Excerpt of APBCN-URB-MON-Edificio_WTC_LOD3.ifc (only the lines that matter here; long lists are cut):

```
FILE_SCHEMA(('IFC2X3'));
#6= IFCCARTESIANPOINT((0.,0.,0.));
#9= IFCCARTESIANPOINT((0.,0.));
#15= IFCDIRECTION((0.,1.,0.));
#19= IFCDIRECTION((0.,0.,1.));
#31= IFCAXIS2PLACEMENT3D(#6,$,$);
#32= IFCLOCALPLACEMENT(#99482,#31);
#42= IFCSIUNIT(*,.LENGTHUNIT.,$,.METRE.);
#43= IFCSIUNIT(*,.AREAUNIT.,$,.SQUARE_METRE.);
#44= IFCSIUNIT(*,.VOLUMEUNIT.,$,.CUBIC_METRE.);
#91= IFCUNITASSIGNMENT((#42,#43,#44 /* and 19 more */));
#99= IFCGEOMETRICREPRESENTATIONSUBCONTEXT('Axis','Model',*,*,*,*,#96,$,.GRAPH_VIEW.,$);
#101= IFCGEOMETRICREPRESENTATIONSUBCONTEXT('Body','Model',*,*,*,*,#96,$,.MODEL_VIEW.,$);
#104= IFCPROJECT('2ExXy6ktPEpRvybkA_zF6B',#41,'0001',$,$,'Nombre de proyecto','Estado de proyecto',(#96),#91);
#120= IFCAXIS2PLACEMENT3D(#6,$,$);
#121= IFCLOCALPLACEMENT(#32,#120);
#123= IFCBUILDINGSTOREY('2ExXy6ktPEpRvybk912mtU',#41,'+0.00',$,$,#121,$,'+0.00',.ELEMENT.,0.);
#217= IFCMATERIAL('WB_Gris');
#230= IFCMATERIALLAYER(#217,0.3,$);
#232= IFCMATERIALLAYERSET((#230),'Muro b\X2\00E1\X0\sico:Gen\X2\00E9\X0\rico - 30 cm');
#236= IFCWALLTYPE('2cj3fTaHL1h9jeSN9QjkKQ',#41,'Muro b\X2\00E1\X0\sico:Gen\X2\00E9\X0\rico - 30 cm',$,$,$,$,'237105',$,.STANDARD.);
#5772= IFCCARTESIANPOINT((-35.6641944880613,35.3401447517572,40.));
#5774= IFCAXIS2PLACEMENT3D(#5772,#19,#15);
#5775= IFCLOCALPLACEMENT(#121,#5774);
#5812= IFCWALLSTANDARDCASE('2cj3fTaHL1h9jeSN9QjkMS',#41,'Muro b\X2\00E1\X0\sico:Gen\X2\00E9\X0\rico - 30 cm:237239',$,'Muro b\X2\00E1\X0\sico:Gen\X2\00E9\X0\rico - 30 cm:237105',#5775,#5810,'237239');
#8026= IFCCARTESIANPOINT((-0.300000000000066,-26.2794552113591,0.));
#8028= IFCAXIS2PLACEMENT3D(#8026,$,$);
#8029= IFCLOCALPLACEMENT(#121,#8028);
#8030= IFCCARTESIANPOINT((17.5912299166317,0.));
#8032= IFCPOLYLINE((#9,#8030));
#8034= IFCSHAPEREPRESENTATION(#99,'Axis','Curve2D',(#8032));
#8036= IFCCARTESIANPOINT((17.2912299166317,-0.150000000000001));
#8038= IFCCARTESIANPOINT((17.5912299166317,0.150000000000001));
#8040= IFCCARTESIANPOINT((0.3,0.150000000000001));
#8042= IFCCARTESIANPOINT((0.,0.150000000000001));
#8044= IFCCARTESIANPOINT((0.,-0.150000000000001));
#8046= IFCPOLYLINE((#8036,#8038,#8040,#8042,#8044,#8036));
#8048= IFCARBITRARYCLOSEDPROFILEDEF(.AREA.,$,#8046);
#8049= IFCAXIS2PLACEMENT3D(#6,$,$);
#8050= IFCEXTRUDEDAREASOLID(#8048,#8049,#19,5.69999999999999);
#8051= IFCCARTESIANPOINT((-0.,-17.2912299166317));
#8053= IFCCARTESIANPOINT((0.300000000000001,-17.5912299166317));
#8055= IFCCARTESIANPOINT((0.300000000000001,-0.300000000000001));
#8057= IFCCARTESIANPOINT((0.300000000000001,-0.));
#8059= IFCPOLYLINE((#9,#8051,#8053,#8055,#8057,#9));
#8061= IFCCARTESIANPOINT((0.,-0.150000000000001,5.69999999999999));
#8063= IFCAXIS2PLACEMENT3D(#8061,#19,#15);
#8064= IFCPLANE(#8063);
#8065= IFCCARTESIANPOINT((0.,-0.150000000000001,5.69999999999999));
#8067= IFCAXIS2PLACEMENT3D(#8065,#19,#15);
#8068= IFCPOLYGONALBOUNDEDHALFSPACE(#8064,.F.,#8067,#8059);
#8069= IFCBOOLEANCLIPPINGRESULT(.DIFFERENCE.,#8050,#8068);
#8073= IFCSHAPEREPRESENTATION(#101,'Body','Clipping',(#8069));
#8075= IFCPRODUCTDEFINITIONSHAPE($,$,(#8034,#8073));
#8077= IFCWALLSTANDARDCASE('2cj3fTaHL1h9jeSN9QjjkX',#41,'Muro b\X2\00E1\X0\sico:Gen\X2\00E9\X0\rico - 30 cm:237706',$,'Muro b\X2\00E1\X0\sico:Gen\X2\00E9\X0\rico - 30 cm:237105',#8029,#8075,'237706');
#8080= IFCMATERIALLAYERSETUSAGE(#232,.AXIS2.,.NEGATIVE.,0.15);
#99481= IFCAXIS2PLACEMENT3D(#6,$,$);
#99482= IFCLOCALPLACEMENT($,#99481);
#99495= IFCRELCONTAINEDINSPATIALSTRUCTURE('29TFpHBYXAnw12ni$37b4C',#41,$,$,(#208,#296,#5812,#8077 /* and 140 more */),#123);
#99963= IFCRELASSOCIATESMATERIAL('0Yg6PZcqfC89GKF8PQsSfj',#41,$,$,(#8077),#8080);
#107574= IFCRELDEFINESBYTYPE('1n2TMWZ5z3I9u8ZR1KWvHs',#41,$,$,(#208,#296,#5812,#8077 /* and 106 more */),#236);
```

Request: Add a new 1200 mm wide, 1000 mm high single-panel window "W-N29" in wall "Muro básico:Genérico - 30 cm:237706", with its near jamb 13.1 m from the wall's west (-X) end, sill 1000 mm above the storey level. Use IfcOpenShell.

```python
import numpy as np
import ifcopenshell
import ifcopenshell.api.feature
import ifcopenshell.api.geometry
import ifcopenshell.api.root
import ifcopenshell.api.spatial
import ifcopenshell.api.type
import ifcopenshell.geom
import ifcopenshell.util.element
import ifcopenshell.util.placement
import ifcopenshell.util.representation
import ifcopenshell.util.shape
import ifcopenshell.util.unit

model = ifcopenshell.open("APBCN-URB-MON-Edificio_WTC_LOD3.ifc")
unit_scale = ifcopenshell.util.unit.calculate_unit_scale(model)
settings = ifcopenshell.geom.settings()


def volume(element):
    """Net volume in cubic metres, openings subtracted."""
    shape = ifcopenshell.geom.create_shape(settings, element)
    return ifcopenshell.util.shape.get_volume(shape.geometry)


wall = model.by_guid("2cj3fTaHL1h9jeSN9QjjkX")
storey = ifcopenshell.util.element.get_container(wall, ifc_class="IfcBuildingStorey")
context = ifcopenshell.util.representation.get_context(model, "Model", "Body", "MODEL_VIEW")
before = volume(wall)

width, height, from_end, sill = 1.2, 1, 13.1, 1  # metres

# The wall runs along its own X axis, and the end named is its -X end.
wall_shape = ifcopenshell.geom.create_shape(settings, wall)
x, y, z = ifcopenshell.util.shape.get_vertices(wall_shape.geometry).T
start = x.min() + from_end
face, thickness = float(y.min()), float(y.max() - y.min())
wall_matrix = ifcopenshell.util.placement.get_local_placement(wall.ObjectPlacement)
level = ifcopenshell.util.placement.get_local_placement(storey.ObjectPlacement)[2, 3]


def in_wall(x, y):
    """Placement at x, y metres in the wall's axes, at sill height."""
    matrix = wall_matrix.copy()
    matrix[:, 3] = wall_matrix @ np.array([x / unit_scale, y / unit_scale, 0.0, 1.0])
    matrix[2, 3] = level + sill / unit_scale
    return matrix


# Opening: a box that overshoots both wall faces by 50 mm.
opening = ifcopenshell.api.root.create_entity(model, ifc_class="IfcOpeningElement")
box = ifcopenshell.api.geometry.add_wall_representation(
    model, context=context, length=width, height=height, thickness=thickness + 0.1
)
ifcopenshell.api.geometry.assign_representation(model, product=opening, representation=box)
ifcopenshell.api.geometry.edit_object_placement(model, product=opening, matrix=in_wall(start, face - 0.05), is_si=False)
ifcopenshell.api.feature.add_feature(model, feature=opening, element=wall)

window = ifcopenshell.api.root.create_entity(model, ifc_class="IfcWindow", name="W-N29")
window.OverallWidth, window.OverallHeight = width / unit_scale, height / unit_scale
body = ifcopenshell.api.geometry.add_window_representation(
    model,
    context=context,
    overall_width=window.OverallWidth,
    overall_height=window.OverallHeight,
    partition_type="SINGLE_PANEL",
)
ifcopenshell.api.geometry.assign_representation(model, product=window, representation=body)
ifcopenshell.api.spatial.assign_container(model, products=[window], relating_structure=storey)
fills = ifcopenshell.api.feature.add_filling(model, opening=opening, element=window)
fills.OwnerHistory = window.OwnerHistory  # required in IFC2X3

# IFC2X3 keeps the operation on the window style.
style = ifcopenshell.api.root.create_entity(model, ifc_class="IfcWindowStyle", name="W-N29")
style.OperationType, style.ConstructionType = "SINGLE_PANEL", "NOTDEFINED"
style.ParameterTakesPrecedence = style.Sizeable = False
ifcopenshell.api.type.assign_type(model, related_objects=[window], relating_type=style)

# Centre the window in the wall's thickness.
ifcopenshell.api.geometry.edit_object_placement(model, product=window, matrix=in_wall(start, face), is_si=False)
window_shape = ifcopenshell.geom.create_shape(settings, window)
depth = ifcopenshell.util.shape.get_vertices(window_shape.geometry)[:, 1]
offset = face + thickness / 2 - (depth.min() + depth.max()) / 2
ifcopenshell.api.geometry.edit_object_placement(model, product=window, matrix=in_wall(start, offset), is_si=False)

after = volume(wall)

print(f"wall volume {before:.3f} -> {after:.3f} m3")

model.write("APBCN-URB-MON-Edificio_WTC_LOD3_rev.ifc")
```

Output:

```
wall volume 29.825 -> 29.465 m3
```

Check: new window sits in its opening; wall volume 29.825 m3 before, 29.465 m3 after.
